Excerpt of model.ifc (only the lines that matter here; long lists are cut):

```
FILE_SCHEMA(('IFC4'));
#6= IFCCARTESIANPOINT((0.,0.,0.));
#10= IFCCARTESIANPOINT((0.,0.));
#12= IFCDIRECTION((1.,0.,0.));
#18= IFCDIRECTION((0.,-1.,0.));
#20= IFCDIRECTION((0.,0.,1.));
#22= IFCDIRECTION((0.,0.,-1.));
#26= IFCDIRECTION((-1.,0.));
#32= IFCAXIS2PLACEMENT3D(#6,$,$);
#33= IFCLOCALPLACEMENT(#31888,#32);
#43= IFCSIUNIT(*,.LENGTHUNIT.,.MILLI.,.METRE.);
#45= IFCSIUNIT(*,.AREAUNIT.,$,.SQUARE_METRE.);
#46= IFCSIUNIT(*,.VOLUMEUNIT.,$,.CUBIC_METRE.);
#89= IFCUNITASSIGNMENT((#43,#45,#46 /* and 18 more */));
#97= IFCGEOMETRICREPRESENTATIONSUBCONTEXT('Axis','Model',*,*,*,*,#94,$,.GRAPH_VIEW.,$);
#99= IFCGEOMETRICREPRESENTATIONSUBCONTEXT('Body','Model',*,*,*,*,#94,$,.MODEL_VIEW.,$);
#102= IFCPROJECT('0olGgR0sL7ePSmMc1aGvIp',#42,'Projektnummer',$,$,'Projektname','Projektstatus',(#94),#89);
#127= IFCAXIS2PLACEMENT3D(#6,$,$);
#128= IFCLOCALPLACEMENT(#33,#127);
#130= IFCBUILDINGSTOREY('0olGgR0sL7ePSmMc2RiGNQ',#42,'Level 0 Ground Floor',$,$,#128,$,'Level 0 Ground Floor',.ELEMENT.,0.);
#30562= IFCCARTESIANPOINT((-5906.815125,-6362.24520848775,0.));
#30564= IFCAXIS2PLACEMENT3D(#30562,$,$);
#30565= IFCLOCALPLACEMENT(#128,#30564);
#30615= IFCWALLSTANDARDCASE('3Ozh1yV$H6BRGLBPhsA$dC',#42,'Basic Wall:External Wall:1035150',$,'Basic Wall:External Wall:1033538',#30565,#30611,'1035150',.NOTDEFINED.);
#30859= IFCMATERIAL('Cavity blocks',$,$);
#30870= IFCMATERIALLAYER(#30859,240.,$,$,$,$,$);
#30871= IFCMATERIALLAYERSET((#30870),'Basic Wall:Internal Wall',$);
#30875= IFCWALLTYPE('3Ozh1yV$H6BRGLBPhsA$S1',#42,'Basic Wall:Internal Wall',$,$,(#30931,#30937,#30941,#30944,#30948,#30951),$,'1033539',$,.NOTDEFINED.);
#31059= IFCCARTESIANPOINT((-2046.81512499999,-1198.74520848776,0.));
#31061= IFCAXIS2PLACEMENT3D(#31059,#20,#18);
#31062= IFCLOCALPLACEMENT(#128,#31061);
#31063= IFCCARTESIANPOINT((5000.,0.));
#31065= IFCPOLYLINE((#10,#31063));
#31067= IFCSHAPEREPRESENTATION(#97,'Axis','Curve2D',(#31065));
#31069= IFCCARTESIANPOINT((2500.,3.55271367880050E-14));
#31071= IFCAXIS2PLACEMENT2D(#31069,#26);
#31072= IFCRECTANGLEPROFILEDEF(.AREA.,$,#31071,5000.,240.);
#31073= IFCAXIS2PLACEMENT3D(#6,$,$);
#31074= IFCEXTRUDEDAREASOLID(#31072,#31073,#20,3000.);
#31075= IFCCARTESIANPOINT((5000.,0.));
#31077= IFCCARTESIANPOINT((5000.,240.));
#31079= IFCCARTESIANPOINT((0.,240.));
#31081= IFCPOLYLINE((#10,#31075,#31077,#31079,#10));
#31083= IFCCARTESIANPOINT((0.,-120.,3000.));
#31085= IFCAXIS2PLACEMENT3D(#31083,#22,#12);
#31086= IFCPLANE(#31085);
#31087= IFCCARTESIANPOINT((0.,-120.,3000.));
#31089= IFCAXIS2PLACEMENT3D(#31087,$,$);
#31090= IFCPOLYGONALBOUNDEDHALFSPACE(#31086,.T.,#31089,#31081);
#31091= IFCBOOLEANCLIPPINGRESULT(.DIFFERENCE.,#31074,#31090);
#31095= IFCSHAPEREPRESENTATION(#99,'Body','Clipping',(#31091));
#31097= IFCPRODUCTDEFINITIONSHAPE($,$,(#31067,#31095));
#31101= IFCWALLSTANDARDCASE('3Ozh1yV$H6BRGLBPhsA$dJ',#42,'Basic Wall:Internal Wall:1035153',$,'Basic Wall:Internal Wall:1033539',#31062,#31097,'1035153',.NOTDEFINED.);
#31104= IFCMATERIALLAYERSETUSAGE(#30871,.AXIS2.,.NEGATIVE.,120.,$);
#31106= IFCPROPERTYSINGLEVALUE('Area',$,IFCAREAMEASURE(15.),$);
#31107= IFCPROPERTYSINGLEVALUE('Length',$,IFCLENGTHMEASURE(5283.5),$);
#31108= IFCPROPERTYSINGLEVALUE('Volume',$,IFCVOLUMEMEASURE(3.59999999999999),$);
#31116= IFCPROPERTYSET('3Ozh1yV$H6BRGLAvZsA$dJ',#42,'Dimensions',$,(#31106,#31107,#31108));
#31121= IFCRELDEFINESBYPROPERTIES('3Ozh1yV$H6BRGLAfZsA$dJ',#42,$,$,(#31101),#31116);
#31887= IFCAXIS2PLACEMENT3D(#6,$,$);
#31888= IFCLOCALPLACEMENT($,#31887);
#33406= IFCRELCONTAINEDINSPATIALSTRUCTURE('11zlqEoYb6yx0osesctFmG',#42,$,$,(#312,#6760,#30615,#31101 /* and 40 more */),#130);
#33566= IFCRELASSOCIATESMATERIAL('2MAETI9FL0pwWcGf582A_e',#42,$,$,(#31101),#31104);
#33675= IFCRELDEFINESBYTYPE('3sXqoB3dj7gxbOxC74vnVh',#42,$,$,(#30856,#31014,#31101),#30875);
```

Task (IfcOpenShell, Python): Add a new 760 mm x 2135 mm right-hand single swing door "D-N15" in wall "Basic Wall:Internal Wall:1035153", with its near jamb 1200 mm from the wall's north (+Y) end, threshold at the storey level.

```python
import numpy as np
import ifcopenshell
import ifcopenshell.api.feature
import ifcopenshell.api.geometry
import ifcopenshell.api.pset
import ifcopenshell.api.root
import ifcopenshell.api.spatial
import ifcopenshell.geom
import ifcopenshell.util.element
import ifcopenshell.util.placement
import ifcopenshell.util.representation
import ifcopenshell.util.shape
import ifcopenshell.util.unit

model = ifcopenshell.open("model.ifc")
unit_scale = ifcopenshell.util.unit.calculate_unit_scale(model)
area_scale = ifcopenshell.util.unit.calculate_unit_scale(model, "AREAUNIT")
volume_scale = ifcopenshell.util.unit.calculate_unit_scale(model, "VOLUMEUNIT")
settings = ifcopenshell.geom.settings()


def volume(element):
    """Net volume in cubic metres, openings subtracted."""
    shape = ifcopenshell.geom.create_shape(settings, element)
    return ifcopenshell.util.shape.get_volume(shape.geometry)


wall = model.by_guid("3Ozh1yV$H6BRGLBPhsA$dJ")
storey = ifcopenshell.util.element.get_container(wall, ifc_class="IfcBuildingStorey")
context = ifcopenshell.util.representation.get_context(model, "Model", "Body", "MODEL_VIEW")
before = volume(wall)

width, height, from_end, sill = 0.76, 2.135, 1.2, 0.0  # metres

# The wall runs along its own X axis, and the end named is its -X end.
wall_shape = ifcopenshell.geom.create_shape(settings, wall)
x, y, z = ifcopenshell.util.shape.get_vertices(wall_shape.geometry).T
start = x.min() + from_end
face, thickness = float(y.min()), float(y.max() - y.min())
wall_matrix = ifcopenshell.util.placement.get_local_placement(wall.ObjectPlacement)
level = ifcopenshell.util.placement.get_local_placement(storey.ObjectPlacement)[2, 3]


def in_wall(x, y):
    """Placement at x, y metres in the wall's axes, at sill height."""
    matrix = wall_matrix.copy()
    matrix[:, 3] = wall_matrix @ np.array([x / unit_scale, y / unit_scale, 0.0, 1.0])
    matrix[2, 3] = level + sill / unit_scale
    return matrix


# Opening: a box that overshoots both wall faces by 50 mm.
opening = ifcopenshell.api.root.create_entity(model, ifc_class="IfcOpeningElement", predefined_type="OPENING")
box = ifcopenshell.api.geometry.add_wall_representation(
    model, context=context, length=width, height=height, thickness=thickness + 0.1
)
ifcopenshell.api.geometry.assign_representation(model, product=opening, representation=box)
ifcopenshell.api.geometry.edit_object_placement(model, product=opening, matrix=in_wall(start, face - 0.05), is_si=False)
ifcopenshell.api.feature.add_feature(model, feature=opening, element=wall)

door = ifcopenshell.api.root.create_entity(model, ifc_class="IfcDoor", name="D-N15", predefined_type="DOOR")
door.OverallWidth, door.OverallHeight = width / unit_scale, height / unit_scale
door.OperationType = "SINGLE_SWING_RIGHT"
body = ifcopenshell.api.geometry.add_door_representation(
    model,
    context=context,
    overall_width=door.OverallWidth,
    overall_height=door.OverallHeight,
    operation_type="SINGLE_SWING_RIGHT",
    lining_properties={"LiningDepth": thickness / unit_scale, "ThresholdDepth": thickness / unit_scale},
)
ifcopenshell.api.geometry.assign_representation(model, product=door, representation=body)
ifcopenshell.api.spatial.assign_container(model, products=[door], relating_structure=storey)
ifcopenshell.api.feature.add_filling(model, opening=opening, element=door)

# The lining spans the wall, so the door starts at the wall face.
ifcopenshell.api.geometry.edit_object_placement(model, product=door, matrix=in_wall(start, face), is_si=False)

after = volume(wall)

# Update the wall's stored quantities.
pset = model.by_id(ifcopenshell.util.element.get_pset(wall, "Dimensions", should_inherit=False)["id"])
ifcopenshell.api.pset.edit_pset(model, pset=pset, properties={
    "Area": model.create_entity("IfcAreaMeasure", after / thickness / area_scale),
    "Volume": model.create_entity("IfcVolumeMeasure", after / volume_scale),
})

print(f"wall volume {before:.3f} -> {after:.3f} m3")

model.write("model_rev.ifc")
```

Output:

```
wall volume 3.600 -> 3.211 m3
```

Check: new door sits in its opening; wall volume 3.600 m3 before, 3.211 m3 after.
